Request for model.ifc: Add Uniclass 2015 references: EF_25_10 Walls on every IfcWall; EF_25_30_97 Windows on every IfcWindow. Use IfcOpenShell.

First a look at what the model holds.

```python
import ifcopenshell

model = ifcopenshell.open("model.ifc")
print(model.schema)
print("classifications:", [c.Name for c in model.by_type("IfcClassification")])
for ifc_class in ("IfcDoor", "IfcRoof", "IfcStair", "IfcWall", "IfcWindow"):
    print(ifc_class, len(model.by_type(ifc_class)))
```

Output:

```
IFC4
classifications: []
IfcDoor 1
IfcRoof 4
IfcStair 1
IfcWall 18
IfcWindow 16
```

```python
import ifcopenshell
import ifcopenshell.api.classification

model = ifcopenshell.open("model.ifc")

system = ifcopenshell.api.classification.add_classification(model, classification="Uniclass 2015")

codes = {
    "IfcWall": ("EF_25_10", "Walls"),
    "IfcWindow": ("EF_25_30_97", "Windows"),
}
for ifc_class, (code, name) in codes.items():
    products = model.by_type(ifc_class)
    ifcopenshell.api.classification.add_reference(
        model, products=products, classification=system, identification=code, name=name
    )
    print(code, len(products))

model.write("model_v2.ifc")
```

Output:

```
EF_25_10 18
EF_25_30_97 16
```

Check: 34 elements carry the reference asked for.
